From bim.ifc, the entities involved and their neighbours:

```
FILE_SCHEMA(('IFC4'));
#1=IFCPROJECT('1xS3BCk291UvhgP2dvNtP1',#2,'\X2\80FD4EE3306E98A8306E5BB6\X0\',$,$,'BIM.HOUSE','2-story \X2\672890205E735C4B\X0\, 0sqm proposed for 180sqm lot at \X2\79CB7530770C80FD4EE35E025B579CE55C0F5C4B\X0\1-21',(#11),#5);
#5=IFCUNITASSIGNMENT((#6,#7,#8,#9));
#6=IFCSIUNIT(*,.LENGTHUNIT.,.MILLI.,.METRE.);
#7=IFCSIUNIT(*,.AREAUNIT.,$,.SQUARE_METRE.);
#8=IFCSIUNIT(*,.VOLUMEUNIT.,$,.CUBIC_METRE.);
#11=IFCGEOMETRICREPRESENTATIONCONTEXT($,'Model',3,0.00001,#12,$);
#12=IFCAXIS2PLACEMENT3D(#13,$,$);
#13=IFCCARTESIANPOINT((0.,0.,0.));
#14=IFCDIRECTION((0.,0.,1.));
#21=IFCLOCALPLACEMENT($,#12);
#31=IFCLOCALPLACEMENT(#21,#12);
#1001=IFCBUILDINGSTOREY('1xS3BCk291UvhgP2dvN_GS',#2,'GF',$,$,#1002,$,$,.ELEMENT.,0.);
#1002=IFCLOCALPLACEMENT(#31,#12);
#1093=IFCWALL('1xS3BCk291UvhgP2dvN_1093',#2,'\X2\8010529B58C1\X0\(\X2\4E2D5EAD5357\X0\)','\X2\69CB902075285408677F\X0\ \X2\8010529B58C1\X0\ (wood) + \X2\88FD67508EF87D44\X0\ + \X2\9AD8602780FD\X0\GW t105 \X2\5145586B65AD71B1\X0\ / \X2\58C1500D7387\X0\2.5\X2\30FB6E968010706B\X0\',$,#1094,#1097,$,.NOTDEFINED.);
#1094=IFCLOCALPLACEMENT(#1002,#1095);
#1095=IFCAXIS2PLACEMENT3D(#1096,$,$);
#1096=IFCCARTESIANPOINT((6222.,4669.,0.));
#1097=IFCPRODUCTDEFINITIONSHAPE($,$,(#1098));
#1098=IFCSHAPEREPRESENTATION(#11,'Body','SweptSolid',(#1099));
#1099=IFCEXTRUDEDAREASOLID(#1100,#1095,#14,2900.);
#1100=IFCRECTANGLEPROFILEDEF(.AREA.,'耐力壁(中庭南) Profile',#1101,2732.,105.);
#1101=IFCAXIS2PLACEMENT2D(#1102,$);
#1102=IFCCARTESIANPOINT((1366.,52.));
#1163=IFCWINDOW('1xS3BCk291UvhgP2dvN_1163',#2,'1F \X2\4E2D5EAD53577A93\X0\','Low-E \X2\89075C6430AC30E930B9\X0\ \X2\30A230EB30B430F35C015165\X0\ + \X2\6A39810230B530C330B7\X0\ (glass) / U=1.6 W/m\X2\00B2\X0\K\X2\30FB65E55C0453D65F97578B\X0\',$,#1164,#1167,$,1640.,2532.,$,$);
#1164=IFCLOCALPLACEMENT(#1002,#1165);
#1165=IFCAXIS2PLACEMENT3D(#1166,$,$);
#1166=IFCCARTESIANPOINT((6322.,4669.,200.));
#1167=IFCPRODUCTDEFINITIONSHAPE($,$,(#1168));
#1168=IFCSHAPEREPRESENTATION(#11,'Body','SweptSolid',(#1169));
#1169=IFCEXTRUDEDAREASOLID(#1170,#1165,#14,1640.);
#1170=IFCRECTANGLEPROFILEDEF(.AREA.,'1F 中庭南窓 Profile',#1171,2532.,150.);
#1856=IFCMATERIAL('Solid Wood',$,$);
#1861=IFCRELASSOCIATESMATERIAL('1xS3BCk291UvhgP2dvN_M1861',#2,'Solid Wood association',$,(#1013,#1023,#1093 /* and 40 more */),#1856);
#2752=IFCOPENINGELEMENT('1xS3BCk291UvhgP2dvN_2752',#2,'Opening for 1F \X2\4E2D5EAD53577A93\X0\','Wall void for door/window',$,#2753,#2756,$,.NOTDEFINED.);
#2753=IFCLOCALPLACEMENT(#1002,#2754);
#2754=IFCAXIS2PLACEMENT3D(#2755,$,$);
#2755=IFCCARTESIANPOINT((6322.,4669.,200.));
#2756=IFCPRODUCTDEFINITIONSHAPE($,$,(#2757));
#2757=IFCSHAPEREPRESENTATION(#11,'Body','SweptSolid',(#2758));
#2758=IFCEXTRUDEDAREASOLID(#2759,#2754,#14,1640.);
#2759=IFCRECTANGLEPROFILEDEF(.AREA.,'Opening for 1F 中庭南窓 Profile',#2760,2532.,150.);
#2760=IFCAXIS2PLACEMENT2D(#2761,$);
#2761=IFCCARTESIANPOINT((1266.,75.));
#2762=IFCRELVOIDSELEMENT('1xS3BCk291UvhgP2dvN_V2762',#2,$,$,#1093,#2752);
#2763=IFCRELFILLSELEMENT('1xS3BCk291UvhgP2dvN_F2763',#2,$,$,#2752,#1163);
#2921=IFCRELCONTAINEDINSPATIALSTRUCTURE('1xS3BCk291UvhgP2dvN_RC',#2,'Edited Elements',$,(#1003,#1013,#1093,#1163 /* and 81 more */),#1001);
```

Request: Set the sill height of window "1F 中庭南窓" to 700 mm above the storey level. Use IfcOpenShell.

```python
import numpy as np
import ifcopenshell
import ifcopenshell.api.geometry
import ifcopenshell.geom
import ifcopenshell.util.element
import ifcopenshell.util.placement
import ifcopenshell.util.shape
import ifcopenshell.util.unit

model = ifcopenshell.open("bim.ifc")
unit_scale = ifcopenshell.util.unit.calculate_unit_scale(model)

window = model.by_guid("1xS3BCk291UvhgP2dvN_1163")
opening = window.FillsVoids[0].RelatingOpeningElement
storey = ifcopenshell.util.element.get_container(window, ifc_class="IfcBuildingStorey")
level = ifcopenshell.util.placement.get_local_placement(storey.ObjectPlacement)[2, 3]

# The opening's origin need not be at the sill, so measure its lowest point.
shape = ifcopenshell.geom.create_shape(ifcopenshell.geom.settings(), opening)
bottom = ifcopenshell.util.shape.get_shape_bottom_elevation(shape, shape.geometry) / unit_scale
dz = level + 0.7 / unit_scale - bottom

shift = np.array([0.0, 0.0, dz])
# The window is not placed relative to its opening, so move both.
for product in (opening, window):
    matrix = ifcopenshell.util.placement.get_local_placement(product.ObjectPlacement)
    matrix[:3, 3] += shift
    ifcopenshell.api.geometry.edit_object_placement(model, product=product, matrix=matrix, is_si=False)

print(f"moved by {dz * unit_scale:+.3f} m")

model.write("bim_edited.ifc")
```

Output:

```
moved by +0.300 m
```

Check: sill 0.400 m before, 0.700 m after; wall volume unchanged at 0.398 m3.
